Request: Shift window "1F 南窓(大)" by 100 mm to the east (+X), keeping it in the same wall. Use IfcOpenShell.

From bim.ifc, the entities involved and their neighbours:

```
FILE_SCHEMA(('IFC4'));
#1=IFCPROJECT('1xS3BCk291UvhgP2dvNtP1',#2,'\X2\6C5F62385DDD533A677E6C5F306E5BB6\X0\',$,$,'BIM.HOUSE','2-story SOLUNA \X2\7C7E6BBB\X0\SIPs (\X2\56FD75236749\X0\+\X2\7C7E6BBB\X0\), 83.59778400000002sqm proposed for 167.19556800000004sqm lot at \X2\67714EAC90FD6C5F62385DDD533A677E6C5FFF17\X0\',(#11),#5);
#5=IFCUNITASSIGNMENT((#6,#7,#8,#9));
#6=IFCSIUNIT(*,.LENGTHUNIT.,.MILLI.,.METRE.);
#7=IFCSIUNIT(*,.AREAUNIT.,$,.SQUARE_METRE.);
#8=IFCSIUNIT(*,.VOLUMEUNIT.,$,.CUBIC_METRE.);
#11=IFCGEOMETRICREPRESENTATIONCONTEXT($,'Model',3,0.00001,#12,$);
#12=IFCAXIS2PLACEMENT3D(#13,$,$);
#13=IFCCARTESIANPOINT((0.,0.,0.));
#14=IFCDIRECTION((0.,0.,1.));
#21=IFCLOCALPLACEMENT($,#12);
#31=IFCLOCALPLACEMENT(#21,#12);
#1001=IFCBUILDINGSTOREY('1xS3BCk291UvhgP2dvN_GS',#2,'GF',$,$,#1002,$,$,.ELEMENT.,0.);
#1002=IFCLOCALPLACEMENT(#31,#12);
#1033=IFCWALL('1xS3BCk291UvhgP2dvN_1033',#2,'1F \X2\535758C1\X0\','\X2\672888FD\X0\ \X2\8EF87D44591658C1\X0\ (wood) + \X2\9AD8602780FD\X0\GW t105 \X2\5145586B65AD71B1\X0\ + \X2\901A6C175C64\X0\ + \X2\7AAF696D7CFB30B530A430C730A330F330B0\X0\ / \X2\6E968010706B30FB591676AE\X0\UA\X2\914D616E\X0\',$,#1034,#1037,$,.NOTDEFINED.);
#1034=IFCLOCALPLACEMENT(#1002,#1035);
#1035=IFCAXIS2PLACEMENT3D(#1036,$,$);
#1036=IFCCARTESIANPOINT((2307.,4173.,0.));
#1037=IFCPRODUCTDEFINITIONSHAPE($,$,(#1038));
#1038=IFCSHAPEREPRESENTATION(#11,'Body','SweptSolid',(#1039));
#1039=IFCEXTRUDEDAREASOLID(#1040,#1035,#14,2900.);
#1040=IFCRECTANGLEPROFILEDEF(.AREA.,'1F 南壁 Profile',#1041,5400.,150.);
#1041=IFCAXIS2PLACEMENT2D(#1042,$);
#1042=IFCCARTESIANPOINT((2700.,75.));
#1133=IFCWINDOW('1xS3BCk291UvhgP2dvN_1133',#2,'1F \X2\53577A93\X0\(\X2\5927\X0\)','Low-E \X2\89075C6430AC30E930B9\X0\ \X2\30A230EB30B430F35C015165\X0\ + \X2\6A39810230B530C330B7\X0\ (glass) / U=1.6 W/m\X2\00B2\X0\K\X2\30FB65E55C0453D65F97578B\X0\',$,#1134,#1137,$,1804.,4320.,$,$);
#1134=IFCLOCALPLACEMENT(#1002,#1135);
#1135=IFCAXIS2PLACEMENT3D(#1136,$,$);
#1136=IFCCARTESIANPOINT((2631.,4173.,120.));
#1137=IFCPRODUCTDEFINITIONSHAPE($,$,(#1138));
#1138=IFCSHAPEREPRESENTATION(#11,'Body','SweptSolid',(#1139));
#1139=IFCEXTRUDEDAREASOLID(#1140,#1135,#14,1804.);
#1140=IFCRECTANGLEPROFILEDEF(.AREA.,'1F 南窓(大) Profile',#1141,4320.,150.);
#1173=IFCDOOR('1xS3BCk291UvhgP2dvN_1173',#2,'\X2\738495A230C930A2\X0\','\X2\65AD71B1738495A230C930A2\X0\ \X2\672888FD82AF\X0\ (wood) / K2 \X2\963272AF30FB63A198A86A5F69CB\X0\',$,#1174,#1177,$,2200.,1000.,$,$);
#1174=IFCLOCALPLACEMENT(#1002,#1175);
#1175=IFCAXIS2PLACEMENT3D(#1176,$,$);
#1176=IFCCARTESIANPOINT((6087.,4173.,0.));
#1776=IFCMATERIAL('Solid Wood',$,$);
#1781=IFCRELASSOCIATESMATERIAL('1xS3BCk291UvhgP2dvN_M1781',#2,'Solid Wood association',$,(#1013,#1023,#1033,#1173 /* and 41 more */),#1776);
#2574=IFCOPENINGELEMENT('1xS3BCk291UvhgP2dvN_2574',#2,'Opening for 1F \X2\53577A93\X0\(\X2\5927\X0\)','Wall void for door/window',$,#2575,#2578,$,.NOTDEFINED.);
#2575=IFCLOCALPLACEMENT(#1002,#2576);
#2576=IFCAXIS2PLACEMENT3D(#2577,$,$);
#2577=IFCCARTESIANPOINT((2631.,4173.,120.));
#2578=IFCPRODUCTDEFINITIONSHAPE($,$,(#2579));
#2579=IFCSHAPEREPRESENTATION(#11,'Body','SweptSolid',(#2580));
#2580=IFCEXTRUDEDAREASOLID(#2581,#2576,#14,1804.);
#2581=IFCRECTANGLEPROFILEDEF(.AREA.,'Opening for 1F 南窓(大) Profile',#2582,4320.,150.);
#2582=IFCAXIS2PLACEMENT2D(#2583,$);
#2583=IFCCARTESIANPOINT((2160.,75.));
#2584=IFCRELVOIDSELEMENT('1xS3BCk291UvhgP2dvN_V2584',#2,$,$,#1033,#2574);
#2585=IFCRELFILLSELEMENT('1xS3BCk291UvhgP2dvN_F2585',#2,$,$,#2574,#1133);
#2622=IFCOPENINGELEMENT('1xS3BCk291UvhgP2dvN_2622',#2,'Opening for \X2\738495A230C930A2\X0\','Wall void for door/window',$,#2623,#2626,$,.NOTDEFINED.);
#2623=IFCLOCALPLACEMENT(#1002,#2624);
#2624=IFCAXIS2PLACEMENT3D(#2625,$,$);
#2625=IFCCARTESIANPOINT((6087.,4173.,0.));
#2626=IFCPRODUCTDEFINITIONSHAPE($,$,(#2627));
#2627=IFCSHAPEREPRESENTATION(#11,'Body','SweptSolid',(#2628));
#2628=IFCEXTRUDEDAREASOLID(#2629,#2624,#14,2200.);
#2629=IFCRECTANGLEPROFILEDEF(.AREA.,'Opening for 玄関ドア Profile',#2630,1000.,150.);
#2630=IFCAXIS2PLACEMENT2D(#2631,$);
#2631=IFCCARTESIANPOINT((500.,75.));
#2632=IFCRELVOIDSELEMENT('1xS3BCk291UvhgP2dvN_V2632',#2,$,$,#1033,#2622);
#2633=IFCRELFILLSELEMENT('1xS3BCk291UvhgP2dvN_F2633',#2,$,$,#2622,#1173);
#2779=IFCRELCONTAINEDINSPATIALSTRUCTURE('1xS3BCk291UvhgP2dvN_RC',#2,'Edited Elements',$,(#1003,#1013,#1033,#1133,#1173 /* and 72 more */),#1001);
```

```python
import ifcopenshell
import ifcopenshell.api.geometry
import ifcopenshell.util.placement
import ifcopenshell.util.unit

model = ifcopenshell.open("bim.ifc")
unit_scale = ifcopenshell.util.unit.calculate_unit_scale(model)

window = model.by_guid("1xS3BCk291UvhgP2dvN_1133")
opening = window.FillsVoids[0].RelatingOpeningElement
wall = opening.VoidsElements[0].RelatingBuildingElement

wall_matrix = ifcopenshell.util.placement.get_local_placement(wall.ObjectPlacement)
shift = wall_matrix[:3, 0] * 0.1 / unit_scale
before = ifcopenshell.util.placement.get_local_placement(window.ObjectPlacement)[:3, 3].copy()

# The window is not placed relative to its opening, so move both.
for product in (opening, window):
    matrix = ifcopenshell.util.placement.get_local_placement(product.ObjectPlacement)
    matrix[:3, 3] += shift
    ifcopenshell.api.geometry.edit_object_placement(model, product=product, matrix=matrix, is_si=False)

after = ifcopenshell.util.placement.get_local_placement(window.ObjectPlacement)[:3, 3]
print("window moved by", (after - before).round(3) + 0.0)

model.write("bim_v2.ifc")
```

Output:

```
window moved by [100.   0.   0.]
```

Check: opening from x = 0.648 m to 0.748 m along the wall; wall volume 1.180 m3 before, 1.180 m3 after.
